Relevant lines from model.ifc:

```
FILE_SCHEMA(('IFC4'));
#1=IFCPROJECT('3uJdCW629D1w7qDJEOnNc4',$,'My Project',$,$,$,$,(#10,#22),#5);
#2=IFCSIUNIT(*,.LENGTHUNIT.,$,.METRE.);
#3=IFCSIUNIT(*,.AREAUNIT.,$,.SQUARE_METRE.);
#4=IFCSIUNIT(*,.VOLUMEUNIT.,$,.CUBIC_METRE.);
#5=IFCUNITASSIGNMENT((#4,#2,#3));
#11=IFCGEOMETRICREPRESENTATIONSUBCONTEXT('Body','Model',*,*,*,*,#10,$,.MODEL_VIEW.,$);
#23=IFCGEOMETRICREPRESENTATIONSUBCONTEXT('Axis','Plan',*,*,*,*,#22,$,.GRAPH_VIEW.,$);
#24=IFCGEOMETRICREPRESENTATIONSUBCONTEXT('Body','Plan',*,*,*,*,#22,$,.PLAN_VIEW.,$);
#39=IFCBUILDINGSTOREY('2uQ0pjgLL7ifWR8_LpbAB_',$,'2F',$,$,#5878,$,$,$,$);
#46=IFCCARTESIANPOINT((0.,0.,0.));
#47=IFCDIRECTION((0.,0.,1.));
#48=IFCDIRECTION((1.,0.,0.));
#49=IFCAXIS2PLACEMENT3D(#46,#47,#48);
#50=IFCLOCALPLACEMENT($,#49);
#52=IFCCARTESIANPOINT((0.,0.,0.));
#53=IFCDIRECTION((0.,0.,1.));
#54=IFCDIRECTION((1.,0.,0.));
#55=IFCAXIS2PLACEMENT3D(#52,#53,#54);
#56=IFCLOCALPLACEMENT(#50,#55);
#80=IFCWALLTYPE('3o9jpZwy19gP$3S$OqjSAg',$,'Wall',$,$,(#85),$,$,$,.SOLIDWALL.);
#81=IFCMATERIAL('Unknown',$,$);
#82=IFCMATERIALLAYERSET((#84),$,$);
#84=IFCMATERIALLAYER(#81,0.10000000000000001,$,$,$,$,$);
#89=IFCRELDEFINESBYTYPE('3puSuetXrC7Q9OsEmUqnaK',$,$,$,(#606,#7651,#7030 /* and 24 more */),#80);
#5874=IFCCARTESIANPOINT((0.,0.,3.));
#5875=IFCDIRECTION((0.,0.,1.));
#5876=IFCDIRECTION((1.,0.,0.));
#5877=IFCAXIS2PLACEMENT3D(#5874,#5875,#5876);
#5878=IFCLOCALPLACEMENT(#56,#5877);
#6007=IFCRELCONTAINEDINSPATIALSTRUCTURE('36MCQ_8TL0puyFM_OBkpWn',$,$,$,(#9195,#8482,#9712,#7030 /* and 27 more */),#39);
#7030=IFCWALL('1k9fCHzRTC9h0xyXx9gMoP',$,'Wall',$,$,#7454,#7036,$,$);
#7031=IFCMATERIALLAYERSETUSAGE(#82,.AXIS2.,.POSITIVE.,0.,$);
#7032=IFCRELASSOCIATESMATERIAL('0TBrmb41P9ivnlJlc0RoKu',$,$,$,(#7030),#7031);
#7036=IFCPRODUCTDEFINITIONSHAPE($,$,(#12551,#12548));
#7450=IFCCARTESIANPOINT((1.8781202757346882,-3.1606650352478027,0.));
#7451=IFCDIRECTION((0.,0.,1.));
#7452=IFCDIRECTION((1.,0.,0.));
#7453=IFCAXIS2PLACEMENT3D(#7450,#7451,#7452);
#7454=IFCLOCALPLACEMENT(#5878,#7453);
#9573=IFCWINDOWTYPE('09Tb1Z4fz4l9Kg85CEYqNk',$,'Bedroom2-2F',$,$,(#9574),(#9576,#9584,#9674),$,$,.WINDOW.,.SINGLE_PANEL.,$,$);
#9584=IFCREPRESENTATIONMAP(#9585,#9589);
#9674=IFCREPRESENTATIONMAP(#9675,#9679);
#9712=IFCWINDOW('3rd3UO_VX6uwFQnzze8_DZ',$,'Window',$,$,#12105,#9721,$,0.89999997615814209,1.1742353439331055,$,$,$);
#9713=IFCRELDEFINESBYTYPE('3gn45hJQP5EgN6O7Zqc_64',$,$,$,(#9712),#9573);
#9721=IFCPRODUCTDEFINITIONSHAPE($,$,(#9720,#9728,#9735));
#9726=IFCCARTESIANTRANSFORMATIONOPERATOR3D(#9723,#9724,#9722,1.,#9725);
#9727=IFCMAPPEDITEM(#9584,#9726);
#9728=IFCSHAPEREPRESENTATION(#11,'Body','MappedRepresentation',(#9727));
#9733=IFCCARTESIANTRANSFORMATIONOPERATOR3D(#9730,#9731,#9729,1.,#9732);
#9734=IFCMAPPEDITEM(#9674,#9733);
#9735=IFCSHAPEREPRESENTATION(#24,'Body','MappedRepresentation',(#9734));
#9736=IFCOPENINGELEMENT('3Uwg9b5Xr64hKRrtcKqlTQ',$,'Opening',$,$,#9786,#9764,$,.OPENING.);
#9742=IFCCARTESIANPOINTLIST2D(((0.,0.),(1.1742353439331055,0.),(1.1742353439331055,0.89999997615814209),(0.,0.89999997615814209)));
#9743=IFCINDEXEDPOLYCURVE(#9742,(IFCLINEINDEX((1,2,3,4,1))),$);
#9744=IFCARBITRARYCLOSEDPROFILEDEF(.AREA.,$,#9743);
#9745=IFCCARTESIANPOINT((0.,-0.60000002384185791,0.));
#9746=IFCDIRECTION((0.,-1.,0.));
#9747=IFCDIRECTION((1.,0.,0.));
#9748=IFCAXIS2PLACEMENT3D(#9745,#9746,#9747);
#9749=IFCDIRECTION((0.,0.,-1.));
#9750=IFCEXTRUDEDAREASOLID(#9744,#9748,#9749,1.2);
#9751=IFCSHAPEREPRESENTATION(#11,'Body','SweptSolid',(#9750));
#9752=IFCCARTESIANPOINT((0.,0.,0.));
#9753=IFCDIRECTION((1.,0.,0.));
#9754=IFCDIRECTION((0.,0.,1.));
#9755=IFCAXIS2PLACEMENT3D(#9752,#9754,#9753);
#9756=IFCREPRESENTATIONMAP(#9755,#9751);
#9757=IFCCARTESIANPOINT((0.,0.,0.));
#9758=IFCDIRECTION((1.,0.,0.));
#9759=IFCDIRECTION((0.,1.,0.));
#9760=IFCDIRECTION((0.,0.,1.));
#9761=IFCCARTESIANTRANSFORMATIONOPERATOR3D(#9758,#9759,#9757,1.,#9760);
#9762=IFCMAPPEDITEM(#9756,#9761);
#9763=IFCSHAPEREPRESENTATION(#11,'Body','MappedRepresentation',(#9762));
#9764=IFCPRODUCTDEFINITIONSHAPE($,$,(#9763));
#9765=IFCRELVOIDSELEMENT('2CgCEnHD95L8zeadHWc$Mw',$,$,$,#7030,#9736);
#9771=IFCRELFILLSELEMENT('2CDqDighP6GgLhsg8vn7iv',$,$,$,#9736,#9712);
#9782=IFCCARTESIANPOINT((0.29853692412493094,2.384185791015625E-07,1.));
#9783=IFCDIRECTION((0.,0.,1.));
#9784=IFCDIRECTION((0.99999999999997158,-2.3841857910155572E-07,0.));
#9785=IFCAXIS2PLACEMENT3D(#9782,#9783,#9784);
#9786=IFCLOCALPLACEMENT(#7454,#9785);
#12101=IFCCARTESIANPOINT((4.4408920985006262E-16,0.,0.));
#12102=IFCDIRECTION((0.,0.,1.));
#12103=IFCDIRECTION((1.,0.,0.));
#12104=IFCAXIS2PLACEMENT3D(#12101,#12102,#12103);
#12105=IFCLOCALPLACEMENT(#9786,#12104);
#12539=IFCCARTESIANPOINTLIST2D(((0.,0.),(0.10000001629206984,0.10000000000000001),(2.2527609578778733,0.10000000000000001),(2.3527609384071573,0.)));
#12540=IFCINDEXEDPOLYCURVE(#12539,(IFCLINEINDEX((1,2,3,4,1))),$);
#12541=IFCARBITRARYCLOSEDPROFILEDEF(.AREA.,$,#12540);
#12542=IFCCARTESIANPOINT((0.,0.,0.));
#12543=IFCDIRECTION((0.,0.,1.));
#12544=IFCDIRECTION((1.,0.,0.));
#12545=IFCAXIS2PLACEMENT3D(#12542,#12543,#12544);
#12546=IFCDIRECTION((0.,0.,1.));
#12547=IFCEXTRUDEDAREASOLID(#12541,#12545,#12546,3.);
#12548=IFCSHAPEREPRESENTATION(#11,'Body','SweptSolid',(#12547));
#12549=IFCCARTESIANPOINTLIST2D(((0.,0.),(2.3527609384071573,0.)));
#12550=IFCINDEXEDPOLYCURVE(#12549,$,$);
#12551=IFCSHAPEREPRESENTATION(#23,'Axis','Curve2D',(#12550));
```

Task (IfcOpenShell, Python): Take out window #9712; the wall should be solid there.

```python
import ifcopenshell
import ifcopenshell.api.feature
import ifcopenshell.api.root
import ifcopenshell.geom
import ifcopenshell.util.shape

model = ifcopenshell.open("model.ifc")
settings = ifcopenshell.geom.settings()


def volume(element):
    """Net volume in cubic metres, openings subtracted."""
    shape = ifcopenshell.geom.create_shape(settings, element)
    return ifcopenshell.util.shape.get_volume(shape.geometry)


window = model.by_id(9712)
opening = window.FillsVoids[0].RelatingOpeningElement
wall = opening.VoidsElements[0].RelatingBuildingElement
before = volume(wall)

ifcopenshell.api.root.remove_product(model, product=window)
ifcopenshell.api.feature.remove_feature(model, feature=opening)

after = volume(wall)

print(f"wall volume {before:.3f} -> {after:.3f} m3")

model.write("model_rev.ifc")
```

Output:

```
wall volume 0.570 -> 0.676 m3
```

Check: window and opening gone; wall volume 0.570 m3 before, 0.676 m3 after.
